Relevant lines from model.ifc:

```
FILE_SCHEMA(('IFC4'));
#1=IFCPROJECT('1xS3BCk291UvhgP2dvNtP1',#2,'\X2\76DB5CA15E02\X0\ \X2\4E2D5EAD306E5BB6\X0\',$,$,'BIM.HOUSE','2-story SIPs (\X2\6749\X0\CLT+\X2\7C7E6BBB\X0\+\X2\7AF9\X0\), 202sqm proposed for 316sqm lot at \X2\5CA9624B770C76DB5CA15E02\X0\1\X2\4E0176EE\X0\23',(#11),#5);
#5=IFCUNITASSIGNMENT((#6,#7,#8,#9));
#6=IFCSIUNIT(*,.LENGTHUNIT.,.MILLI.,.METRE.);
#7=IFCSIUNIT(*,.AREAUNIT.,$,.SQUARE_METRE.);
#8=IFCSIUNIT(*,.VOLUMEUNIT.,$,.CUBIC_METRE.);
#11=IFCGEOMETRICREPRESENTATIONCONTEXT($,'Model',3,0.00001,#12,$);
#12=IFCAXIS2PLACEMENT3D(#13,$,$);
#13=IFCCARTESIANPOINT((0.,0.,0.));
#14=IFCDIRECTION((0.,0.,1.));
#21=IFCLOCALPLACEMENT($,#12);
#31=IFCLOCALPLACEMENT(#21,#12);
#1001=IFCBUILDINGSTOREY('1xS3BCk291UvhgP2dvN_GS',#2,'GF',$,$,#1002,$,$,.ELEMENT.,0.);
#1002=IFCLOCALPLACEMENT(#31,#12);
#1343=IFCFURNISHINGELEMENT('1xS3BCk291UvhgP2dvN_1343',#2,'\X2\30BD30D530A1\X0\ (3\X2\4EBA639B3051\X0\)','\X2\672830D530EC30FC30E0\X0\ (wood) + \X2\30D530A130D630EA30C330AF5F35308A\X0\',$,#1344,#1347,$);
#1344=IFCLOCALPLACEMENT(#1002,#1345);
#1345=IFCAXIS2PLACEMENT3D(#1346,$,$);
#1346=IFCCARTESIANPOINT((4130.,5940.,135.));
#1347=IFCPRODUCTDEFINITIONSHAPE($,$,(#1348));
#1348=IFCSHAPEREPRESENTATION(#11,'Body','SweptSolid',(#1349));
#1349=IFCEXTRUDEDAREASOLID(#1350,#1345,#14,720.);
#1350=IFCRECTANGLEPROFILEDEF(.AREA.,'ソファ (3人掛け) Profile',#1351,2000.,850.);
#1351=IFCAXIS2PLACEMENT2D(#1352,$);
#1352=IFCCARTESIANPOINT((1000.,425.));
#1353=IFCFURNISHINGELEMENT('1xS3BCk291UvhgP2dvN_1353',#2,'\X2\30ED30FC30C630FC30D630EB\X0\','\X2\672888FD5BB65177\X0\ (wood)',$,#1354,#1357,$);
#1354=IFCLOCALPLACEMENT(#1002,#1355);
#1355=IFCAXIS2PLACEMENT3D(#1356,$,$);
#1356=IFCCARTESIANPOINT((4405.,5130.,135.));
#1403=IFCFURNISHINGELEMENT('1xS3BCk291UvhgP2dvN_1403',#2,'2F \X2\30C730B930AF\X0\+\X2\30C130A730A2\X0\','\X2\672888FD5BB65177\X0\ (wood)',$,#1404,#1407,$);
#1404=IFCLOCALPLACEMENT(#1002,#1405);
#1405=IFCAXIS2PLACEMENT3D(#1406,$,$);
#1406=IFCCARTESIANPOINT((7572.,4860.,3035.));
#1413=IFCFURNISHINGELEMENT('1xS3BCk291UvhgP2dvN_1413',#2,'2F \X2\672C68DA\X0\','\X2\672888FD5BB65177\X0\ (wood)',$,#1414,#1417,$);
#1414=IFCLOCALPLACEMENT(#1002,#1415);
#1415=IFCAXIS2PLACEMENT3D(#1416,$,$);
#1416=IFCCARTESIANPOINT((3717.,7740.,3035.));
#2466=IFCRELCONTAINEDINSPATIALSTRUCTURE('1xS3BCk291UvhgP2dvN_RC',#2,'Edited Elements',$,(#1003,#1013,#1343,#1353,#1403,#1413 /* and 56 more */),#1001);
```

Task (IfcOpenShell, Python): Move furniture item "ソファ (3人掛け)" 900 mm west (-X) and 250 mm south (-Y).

```python
import ifcopenshell
import ifcopenshell.api.geometry
import ifcopenshell.util.placement
import ifcopenshell.util.unit

model = ifcopenshell.open("model.ifc")
unit_scale = ifcopenshell.util.unit.calculate_unit_scale(model)

item = model.by_guid("1xS3BCk291UvhgP2dvN_1343")
matrix = ifcopenshell.util.placement.get_local_placement(item.ObjectPlacement)
matrix[0, 3] -= 0.9 / unit_scale
matrix[1, 3] -= 0.25 / unit_scale
ifcopenshell.api.geometry.edit_object_placement(model, product=item, matrix=matrix, is_si=False)

print(ifcopenshell.util.placement.get_local_placement(item.ObjectPlacement).round(3) + 0.0)

model.write("model_v2.ifc")
```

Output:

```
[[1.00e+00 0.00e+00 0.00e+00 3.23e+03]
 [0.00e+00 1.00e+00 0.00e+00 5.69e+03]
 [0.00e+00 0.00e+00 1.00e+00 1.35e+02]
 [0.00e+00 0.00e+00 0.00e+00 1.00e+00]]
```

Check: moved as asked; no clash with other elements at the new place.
